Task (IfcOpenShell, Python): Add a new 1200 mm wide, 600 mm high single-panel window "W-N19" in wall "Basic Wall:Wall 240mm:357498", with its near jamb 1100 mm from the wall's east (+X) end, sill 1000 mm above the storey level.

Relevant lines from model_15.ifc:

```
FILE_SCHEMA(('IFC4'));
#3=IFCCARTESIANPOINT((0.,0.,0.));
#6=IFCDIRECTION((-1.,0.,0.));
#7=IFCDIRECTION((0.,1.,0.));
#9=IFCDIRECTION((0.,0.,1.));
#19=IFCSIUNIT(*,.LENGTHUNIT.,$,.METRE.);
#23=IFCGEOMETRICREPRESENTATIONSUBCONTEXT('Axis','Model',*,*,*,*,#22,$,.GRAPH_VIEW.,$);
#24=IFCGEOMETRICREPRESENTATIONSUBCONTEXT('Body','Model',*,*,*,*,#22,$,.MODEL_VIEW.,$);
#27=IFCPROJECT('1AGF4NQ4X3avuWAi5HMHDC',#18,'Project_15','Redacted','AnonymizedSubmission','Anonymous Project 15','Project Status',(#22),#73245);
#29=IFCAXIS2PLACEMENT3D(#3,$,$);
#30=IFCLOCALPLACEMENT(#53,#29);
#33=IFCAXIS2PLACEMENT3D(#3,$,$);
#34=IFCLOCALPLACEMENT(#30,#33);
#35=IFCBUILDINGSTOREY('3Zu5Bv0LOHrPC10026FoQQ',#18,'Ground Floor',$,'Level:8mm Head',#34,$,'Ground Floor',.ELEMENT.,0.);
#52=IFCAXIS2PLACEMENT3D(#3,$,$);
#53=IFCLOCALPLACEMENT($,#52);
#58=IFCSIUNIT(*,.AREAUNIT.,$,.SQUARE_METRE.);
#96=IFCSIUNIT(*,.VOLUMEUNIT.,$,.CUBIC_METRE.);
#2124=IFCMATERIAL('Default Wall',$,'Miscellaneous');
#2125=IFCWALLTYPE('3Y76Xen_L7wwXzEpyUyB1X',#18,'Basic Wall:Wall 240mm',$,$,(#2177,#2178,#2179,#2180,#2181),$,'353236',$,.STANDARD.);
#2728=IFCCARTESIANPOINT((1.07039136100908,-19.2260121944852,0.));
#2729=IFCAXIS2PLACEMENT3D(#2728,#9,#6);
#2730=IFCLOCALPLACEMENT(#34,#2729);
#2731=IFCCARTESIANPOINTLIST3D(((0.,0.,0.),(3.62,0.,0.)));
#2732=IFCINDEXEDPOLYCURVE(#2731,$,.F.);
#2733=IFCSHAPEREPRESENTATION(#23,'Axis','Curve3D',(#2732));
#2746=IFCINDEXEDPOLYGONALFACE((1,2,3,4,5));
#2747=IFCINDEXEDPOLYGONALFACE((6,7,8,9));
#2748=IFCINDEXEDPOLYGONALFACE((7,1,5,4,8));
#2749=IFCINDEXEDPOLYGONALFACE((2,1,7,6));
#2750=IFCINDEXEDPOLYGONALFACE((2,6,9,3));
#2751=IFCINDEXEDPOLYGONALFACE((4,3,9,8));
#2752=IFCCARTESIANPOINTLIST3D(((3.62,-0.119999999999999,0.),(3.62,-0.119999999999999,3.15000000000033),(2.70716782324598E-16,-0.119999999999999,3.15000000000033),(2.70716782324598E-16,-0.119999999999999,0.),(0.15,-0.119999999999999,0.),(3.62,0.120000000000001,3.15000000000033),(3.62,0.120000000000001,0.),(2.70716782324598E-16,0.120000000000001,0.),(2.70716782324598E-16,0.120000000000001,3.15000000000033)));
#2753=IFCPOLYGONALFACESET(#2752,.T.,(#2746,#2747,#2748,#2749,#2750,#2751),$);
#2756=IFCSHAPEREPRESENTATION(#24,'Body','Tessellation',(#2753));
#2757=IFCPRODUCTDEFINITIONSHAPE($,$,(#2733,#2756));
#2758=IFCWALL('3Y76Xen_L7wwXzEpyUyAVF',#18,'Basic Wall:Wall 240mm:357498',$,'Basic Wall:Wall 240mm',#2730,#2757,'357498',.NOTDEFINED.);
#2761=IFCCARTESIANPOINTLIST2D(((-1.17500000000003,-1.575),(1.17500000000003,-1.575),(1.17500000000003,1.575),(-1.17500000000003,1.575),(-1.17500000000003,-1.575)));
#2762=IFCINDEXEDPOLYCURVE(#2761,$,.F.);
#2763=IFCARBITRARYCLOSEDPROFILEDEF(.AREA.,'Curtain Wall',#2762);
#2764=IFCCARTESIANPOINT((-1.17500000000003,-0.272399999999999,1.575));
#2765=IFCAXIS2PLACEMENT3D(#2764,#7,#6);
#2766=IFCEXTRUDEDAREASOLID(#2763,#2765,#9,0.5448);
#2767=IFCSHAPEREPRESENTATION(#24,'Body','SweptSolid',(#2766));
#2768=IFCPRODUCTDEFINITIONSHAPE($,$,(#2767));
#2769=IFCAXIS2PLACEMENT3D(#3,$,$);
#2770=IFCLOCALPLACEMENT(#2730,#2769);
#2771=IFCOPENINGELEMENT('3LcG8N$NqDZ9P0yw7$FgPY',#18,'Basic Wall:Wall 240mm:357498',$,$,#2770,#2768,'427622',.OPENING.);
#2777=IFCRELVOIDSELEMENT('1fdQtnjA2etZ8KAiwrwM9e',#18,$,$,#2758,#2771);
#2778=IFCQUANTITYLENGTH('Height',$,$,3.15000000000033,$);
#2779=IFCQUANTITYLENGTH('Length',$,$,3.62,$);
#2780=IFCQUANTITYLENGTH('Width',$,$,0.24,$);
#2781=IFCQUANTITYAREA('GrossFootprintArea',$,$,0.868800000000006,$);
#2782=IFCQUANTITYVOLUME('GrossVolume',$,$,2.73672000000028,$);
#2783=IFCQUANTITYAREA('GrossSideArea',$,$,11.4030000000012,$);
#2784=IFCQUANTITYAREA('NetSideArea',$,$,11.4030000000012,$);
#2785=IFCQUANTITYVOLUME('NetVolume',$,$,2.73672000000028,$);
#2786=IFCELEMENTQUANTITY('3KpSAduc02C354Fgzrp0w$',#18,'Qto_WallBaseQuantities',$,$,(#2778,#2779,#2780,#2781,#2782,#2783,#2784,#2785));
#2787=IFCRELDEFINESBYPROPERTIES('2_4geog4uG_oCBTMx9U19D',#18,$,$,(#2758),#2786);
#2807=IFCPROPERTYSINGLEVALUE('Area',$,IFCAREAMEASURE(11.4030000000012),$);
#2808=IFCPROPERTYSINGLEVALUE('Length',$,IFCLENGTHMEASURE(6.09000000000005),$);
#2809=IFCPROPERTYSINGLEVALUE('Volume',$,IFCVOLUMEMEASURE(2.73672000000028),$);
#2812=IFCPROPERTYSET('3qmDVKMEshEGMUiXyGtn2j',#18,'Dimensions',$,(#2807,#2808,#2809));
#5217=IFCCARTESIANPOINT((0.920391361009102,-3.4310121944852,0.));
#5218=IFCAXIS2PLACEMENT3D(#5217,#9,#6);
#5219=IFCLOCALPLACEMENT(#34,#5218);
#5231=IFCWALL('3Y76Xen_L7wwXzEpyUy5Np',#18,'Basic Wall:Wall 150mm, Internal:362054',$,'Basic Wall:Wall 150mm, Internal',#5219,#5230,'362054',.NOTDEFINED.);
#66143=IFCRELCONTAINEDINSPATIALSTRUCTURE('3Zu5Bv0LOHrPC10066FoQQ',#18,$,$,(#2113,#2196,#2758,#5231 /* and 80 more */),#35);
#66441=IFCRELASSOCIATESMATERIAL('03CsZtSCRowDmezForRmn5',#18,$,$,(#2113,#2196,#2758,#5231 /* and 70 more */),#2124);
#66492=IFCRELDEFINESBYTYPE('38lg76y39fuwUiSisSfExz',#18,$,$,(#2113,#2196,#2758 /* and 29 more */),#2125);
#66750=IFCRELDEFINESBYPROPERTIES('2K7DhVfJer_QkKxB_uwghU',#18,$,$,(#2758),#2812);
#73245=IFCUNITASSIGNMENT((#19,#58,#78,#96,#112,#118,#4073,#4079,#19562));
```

```python
import numpy as np
import ifcopenshell
import ifcopenshell.api.feature
import ifcopenshell.api.geometry
import ifcopenshell.api.pset
import ifcopenshell.api.root
import ifcopenshell.api.spatial
import ifcopenshell.geom
import ifcopenshell.util.element
import ifcopenshell.util.placement
import ifcopenshell.util.representation
import ifcopenshell.util.shape
import ifcopenshell.util.unit

model = ifcopenshell.open("model_15.ifc")
unit_scale = ifcopenshell.util.unit.calculate_unit_scale(model)
area_scale = ifcopenshell.util.unit.calculate_unit_scale(model, "AREAUNIT")
volume_scale = ifcopenshell.util.unit.calculate_unit_scale(model, "VOLUMEUNIT")
settings = ifcopenshell.geom.settings()


def volume(element):
    """Net volume in cubic metres, openings subtracted."""
    shape = ifcopenshell.geom.create_shape(settings, element)
    return ifcopenshell.util.shape.get_volume(shape.geometry)


wall = model.by_guid("3Y76Xen_L7wwXzEpyUyAVF")
storey = ifcopenshell.util.element.get_container(wall, ifc_class="IfcBuildingStorey")
context = ifcopenshell.util.representation.get_context(model, "Model", "Body", "MODEL_VIEW")
before = volume(wall)

width, height, from_end, sill = 1.2, 0.6, 1.1, 1  # metres

# The wall runs along its own X axis, and the end named is its -X end.
wall_shape = ifcopenshell.geom.create_shape(settings, wall)
x, y, z = ifcopenshell.util.shape.get_vertices(wall_shape.geometry).T
start = x.min() + from_end
face, thickness = float(y.min()), float(y.max() - y.min())
wall_matrix = ifcopenshell.util.placement.get_local_placement(wall.ObjectPlacement)
level = ifcopenshell.util.placement.get_local_placement(storey.ObjectPlacement)[2, 3]


def in_wall(x, y):
    """Placement at x, y metres in the wall's axes, at sill height."""
    matrix = wall_matrix.copy()
    matrix[:, 3] = wall_matrix @ np.array([x / unit_scale, y / unit_scale, 0.0, 1.0])
    matrix[2, 3] = level + sill / unit_scale
    return matrix


# Opening: a box that overshoots both wall faces by 50 mm.
opening = ifcopenshell.api.root.create_entity(model, ifc_class="IfcOpeningElement", predefined_type="OPENING")
box = ifcopenshell.api.geometry.add_wall_representation(
    model, context=context, length=width, height=height, thickness=thickness + 0.1
)
ifcopenshell.api.geometry.assign_representation(model, product=opening, representation=box)
ifcopenshell.api.geometry.edit_object_placement(model, product=opening, matrix=in_wall(start, face - 0.05), is_si=False)
ifcopenshell.api.feature.add_feature(model, feature=opening, element=wall)

window = ifcopenshell.api.root.create_entity(model, ifc_class="IfcWindow", name="W-N19", predefined_type="WINDOW")
window.OverallWidth, window.OverallHeight = width / unit_scale, height / unit_scale
window.PartitioningType = "SINGLE_PANEL"
body = ifcopenshell.api.geometry.add_window_representation(
    model,
    context=context,
    overall_width=window.OverallWidth,
    overall_height=window.OverallHeight,
    partition_type="SINGLE_PANEL",
)
ifcopenshell.api.geometry.assign_representation(model, product=window, representation=body)
ifcopenshell.api.spatial.assign_container(model, products=[window], relating_structure=storey)
ifcopenshell.api.feature.add_filling(model, opening=opening, element=window)

# Centre the window in the wall's thickness.
ifcopenshell.api.geometry.edit_object_placement(model, product=window, matrix=in_wall(start, face), is_si=False)
window_shape = ifcopenshell.geom.create_shape(settings, window)
depth = ifcopenshell.util.shape.get_vertices(window_shape.geometry)[:, 1]
offset = face + thickness / 2 - (depth.min() + depth.max()) / 2
ifcopenshell.api.geometry.edit_object_placement(model, product=window, matrix=in_wall(start, offset), is_si=False)

after = volume(wall)

# Update the wall's stored quantities.
qto = model.by_id(ifcopenshell.util.element.get_pset(wall, "Qto_WallBaseQuantities", should_inherit=False)["id"])
ifcopenshell.api.pset.edit_qto(model, qto=qto, properties={
    "NetSideArea": after / thickness / area_scale,
    "NetVolume": after / volume_scale,
})
pset = model.by_id(ifcopenshell.util.element.get_pset(wall, "Dimensions", should_inherit=False)["id"])
ifcopenshell.api.pset.edit_pset(model, pset=pset, properties={
    "Area": model.create_entity("IfcAreaMeasure", after / thickness / area_scale),
    "Volume": model.create_entity("IfcVolumeMeasure", after / volume_scale),
})

print(f"wall volume {before:.3f} -> {after:.3f} m3")

model.write("model_15_updated.ifc")
```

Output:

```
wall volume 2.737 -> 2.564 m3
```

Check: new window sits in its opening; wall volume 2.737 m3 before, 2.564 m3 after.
